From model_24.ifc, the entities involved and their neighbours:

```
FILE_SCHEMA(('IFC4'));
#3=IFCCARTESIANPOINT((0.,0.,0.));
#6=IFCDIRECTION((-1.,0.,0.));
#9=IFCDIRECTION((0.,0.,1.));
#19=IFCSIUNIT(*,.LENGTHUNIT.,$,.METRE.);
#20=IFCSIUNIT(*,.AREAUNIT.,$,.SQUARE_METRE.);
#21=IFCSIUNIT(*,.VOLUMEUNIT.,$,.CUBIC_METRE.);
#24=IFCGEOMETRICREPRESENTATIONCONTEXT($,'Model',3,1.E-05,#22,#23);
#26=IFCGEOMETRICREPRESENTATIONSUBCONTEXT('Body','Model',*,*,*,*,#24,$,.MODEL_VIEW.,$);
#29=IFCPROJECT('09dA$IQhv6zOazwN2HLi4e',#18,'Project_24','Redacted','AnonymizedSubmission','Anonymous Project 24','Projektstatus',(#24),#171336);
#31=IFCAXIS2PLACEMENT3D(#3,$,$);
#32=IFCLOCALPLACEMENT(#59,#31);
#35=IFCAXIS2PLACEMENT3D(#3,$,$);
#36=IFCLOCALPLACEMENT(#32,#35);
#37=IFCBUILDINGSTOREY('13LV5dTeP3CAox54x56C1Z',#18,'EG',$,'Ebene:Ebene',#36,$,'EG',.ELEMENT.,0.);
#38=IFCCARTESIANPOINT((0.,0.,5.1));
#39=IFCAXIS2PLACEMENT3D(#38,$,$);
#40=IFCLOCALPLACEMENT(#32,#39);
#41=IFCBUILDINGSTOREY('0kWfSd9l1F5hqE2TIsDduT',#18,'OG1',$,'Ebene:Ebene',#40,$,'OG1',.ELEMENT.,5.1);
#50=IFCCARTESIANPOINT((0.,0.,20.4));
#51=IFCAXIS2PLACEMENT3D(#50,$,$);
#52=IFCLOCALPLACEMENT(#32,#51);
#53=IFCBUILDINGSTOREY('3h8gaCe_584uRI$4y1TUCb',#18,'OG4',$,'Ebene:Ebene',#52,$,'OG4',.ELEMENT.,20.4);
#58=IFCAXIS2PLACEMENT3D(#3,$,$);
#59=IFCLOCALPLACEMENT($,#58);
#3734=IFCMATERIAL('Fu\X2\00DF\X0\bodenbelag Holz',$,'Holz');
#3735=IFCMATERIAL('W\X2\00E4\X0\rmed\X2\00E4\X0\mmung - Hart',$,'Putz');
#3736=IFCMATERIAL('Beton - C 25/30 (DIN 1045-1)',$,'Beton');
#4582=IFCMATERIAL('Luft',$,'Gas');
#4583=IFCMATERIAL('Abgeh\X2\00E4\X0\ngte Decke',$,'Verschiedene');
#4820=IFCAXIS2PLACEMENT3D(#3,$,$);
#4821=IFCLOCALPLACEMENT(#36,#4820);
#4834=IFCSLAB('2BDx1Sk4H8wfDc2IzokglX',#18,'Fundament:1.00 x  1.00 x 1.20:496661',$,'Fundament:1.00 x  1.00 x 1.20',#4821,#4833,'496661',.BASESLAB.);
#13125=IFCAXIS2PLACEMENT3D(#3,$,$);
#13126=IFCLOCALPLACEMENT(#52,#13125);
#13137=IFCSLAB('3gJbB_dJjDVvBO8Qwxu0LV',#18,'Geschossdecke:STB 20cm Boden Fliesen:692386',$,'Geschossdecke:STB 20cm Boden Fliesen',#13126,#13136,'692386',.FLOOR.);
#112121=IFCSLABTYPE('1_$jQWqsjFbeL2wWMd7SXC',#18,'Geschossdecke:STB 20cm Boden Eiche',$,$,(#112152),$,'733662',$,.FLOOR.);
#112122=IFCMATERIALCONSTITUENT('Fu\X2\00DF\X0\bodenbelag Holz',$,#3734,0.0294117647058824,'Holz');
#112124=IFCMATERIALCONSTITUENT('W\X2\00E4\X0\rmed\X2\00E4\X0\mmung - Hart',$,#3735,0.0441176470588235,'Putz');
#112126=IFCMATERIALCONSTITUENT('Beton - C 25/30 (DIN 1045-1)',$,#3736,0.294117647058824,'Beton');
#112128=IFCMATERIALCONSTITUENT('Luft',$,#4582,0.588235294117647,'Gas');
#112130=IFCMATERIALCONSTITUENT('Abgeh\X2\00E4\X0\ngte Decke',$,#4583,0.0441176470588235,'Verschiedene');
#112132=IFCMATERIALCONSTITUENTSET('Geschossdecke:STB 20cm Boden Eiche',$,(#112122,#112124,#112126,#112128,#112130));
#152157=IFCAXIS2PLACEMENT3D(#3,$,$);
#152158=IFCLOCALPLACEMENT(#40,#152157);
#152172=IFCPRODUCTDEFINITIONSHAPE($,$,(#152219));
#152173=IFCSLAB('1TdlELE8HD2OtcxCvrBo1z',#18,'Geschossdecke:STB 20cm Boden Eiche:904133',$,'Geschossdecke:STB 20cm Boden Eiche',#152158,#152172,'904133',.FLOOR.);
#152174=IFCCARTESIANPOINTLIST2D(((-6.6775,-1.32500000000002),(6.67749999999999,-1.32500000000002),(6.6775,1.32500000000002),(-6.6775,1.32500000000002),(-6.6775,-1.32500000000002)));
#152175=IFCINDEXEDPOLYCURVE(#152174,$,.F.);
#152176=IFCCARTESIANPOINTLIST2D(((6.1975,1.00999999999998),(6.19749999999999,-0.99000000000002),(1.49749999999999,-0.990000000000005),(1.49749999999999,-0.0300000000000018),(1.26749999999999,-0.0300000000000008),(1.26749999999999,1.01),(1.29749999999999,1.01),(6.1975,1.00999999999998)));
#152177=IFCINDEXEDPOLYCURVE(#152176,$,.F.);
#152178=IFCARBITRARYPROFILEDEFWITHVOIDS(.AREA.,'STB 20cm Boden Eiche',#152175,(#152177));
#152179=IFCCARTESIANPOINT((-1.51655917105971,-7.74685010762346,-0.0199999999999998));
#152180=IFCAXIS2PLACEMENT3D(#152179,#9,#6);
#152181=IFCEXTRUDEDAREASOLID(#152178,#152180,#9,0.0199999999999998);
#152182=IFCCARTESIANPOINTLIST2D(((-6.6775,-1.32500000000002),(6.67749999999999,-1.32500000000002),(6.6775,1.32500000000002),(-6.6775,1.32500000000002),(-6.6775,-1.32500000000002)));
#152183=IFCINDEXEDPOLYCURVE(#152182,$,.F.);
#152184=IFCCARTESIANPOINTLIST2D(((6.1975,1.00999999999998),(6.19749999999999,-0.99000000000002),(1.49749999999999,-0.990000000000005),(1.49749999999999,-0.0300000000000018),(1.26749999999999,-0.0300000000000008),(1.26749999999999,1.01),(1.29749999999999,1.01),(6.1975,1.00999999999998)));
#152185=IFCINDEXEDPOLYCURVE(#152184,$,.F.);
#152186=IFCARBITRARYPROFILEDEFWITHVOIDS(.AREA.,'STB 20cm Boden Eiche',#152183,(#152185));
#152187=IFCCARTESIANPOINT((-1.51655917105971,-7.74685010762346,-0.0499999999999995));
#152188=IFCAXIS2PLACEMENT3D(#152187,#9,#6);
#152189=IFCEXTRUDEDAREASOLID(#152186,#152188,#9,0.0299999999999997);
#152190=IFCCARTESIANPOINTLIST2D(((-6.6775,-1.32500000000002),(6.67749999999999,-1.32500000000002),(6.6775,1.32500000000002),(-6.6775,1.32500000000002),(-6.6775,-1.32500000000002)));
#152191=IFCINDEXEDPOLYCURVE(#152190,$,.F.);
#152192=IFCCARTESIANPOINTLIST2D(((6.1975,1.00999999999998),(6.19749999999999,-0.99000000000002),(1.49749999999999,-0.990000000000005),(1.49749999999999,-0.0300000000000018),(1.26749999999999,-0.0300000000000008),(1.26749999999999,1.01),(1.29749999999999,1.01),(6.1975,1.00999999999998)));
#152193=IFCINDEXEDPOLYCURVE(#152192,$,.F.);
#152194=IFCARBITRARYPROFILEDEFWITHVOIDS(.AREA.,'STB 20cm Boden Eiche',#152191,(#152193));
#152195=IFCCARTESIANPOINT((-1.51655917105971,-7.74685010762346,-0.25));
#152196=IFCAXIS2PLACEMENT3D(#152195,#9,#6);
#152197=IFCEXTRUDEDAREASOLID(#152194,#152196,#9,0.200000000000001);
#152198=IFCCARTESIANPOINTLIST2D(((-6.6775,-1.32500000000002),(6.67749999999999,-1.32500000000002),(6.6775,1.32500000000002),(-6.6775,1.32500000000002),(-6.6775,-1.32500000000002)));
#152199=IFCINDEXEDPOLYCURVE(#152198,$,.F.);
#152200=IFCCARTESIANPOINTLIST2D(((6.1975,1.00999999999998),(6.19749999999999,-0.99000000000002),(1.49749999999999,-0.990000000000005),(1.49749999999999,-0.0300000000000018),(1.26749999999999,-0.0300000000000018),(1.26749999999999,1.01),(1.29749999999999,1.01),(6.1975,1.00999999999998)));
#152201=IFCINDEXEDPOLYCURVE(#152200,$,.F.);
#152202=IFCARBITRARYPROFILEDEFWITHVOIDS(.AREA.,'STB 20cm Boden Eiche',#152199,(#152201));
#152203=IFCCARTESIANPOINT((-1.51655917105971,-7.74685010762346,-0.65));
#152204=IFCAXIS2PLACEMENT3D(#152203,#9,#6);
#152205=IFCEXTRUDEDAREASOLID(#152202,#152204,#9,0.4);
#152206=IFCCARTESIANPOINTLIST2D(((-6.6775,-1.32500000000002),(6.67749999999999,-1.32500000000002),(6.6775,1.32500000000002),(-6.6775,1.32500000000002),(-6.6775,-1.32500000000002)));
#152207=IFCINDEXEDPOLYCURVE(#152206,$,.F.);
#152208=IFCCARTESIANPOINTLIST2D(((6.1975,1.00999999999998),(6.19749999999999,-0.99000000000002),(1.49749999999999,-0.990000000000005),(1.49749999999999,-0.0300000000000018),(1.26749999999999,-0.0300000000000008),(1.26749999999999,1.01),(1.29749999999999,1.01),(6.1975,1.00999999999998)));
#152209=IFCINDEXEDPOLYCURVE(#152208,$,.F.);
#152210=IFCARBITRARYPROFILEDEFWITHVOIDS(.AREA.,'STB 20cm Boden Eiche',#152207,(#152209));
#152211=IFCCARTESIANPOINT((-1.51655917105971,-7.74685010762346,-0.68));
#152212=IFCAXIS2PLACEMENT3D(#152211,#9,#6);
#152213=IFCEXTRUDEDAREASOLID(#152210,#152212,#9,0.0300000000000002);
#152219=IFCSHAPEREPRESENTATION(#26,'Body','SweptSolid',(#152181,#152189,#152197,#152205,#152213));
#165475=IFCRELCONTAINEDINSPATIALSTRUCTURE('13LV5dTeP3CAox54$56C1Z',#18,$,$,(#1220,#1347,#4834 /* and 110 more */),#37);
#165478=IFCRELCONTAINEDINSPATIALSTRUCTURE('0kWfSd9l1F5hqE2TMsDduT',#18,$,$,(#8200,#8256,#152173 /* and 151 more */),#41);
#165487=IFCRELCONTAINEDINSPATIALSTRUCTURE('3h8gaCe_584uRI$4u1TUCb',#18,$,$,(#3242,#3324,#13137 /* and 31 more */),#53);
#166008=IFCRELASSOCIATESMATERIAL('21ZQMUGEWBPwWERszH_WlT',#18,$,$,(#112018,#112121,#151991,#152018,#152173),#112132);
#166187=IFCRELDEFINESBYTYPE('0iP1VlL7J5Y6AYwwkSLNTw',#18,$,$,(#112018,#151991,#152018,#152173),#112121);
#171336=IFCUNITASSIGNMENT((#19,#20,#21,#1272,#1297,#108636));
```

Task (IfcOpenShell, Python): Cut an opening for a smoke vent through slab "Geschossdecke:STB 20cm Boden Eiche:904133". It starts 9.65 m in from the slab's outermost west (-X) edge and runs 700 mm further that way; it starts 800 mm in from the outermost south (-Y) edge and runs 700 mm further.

```python
import numpy as np
import ifcopenshell
import ifcopenshell.api.feature
import ifcopenshell.api.geometry
import ifcopenshell.api.root
import ifcopenshell.geom
import ifcopenshell.util.placement
import ifcopenshell.util.representation
import ifcopenshell.util.shape
import ifcopenshell.util.unit

model = ifcopenshell.open("model_24.ifc")
unit_scale = ifcopenshell.util.unit.calculate_unit_scale(model)
settings = ifcopenshell.geom.settings()


def volume(element):
    """Net volume in cubic metres, openings subtracted."""
    shape = ifcopenshell.geom.create_shape(settings, element)
    return ifcopenshell.util.shape.get_volume(shape.geometry)


slab = model.by_guid("1TdlELE8HD2OtcxCvrBo1z")
before = volume(slab)

# Extent in the slab's own axes, in metres. The edges named are its -X and -Y sides.
slab_shape = ifcopenshell.geom.create_shape(settings, slab)
vertices = ifcopenshell.util.shape.get_vertices(slab_shape.geometry)
x_min, y_min, bottom = vertices.min(axis=0)
top = vertices[:, 2].max()

opening = ifcopenshell.api.root.create_entity(model, ifc_class="IfcOpeningElement", name="Smoke vent opening", predefined_type="OPENING")
context = ifcopenshell.util.representation.get_context(model, "Model", "Body", "MODEL_VIEW")
width, depth = 0.7, 0.7
outline = [(0.0, 0.0), (width, 0.0), (width, depth), (0.0, depth), (0.0, 0.0)]
# Overshoot both faces by 50 mm so the cut is clean.
shape = ifcopenshell.api.geometry.add_slab_representation(
    model, context=context, depth=top - bottom + 0.1, polyline=outline
)
ifcopenshell.api.geometry.assign_representation(model, product=opening, representation=shape)

matrix = ifcopenshell.util.placement.get_local_placement(slab.ObjectPlacement)
matrix[:, 3] = matrix @ np.append(np.array([x_min + 9.65, y_min + 0.8, bottom - 0.05]) / unit_scale, 1.0)
ifcopenshell.api.geometry.edit_object_placement(model, product=opening, matrix=matrix, is_si=False)
ifcopenshell.api.feature.add_feature(model, feature=opening, element=slab)

after = volume(slab)

print(f"slab volume {before:.3f} -> {after:.3f} m3")

model.write("model_24_rev.ifc")
```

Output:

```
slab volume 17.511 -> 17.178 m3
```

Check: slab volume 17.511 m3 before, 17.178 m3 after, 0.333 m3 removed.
